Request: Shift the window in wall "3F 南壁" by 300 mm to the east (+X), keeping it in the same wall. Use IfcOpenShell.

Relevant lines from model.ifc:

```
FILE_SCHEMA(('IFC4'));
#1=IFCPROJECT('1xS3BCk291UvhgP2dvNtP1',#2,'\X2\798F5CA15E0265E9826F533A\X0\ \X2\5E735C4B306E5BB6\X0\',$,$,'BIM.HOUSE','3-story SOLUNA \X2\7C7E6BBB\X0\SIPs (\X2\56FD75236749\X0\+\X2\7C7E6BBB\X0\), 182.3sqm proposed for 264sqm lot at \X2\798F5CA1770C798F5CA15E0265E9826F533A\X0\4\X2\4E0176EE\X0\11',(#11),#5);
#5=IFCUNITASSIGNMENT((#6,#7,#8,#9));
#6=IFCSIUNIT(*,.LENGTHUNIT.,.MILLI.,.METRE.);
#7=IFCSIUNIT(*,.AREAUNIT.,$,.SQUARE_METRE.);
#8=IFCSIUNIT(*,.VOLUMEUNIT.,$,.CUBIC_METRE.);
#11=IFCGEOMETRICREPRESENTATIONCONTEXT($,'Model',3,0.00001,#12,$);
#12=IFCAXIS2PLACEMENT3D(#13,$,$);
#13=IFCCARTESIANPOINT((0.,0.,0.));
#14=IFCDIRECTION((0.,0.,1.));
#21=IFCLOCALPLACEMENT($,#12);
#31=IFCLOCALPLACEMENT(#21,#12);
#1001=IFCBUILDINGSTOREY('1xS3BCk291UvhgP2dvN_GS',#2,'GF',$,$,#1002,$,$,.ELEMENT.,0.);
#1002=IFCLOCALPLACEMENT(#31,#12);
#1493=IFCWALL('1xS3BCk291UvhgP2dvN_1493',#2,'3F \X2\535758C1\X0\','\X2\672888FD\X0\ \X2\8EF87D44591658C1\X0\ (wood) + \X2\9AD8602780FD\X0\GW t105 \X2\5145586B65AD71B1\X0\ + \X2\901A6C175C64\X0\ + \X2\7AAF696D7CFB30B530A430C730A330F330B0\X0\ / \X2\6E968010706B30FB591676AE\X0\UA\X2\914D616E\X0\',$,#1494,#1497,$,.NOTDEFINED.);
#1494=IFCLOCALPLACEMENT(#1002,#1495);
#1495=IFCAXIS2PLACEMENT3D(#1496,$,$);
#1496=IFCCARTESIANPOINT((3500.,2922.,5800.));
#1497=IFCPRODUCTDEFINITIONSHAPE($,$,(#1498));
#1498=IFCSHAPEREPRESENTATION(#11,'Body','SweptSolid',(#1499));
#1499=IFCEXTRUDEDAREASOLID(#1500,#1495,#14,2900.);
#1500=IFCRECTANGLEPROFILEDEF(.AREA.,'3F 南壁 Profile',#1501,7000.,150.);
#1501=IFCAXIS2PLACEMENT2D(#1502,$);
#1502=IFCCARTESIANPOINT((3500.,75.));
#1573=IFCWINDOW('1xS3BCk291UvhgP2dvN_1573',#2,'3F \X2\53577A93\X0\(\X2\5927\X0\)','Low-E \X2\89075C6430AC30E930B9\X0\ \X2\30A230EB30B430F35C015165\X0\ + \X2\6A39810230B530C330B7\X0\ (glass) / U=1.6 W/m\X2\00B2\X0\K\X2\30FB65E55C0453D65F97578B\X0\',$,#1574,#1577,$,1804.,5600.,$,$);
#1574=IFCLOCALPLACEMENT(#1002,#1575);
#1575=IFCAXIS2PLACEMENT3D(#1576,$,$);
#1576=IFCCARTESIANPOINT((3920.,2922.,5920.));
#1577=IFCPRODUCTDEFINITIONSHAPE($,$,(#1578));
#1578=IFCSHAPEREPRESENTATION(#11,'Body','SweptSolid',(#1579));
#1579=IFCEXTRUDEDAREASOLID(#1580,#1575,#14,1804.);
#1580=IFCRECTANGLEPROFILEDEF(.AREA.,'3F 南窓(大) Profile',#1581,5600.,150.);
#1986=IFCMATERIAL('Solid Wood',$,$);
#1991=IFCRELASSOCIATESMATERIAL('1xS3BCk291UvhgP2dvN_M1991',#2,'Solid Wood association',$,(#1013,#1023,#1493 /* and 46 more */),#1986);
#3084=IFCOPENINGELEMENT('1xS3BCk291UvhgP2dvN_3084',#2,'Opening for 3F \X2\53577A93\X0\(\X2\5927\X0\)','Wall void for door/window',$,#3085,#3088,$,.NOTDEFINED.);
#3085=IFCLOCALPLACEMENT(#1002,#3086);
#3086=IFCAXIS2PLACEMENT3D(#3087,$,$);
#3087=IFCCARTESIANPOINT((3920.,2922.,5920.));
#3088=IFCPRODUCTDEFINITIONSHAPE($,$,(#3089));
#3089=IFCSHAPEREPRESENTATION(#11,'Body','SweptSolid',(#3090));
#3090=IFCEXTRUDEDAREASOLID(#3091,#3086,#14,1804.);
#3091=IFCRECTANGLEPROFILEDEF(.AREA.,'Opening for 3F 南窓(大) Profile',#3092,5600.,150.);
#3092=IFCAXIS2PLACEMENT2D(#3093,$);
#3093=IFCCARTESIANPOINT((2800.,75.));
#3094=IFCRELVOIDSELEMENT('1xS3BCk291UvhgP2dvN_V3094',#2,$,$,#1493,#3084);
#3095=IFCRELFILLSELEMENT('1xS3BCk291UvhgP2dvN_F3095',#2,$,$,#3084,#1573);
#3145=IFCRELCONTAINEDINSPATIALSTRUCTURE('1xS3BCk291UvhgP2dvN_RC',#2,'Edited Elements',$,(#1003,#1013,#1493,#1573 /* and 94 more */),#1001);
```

```python
import ifcopenshell
import ifcopenshell.api.geometry
import ifcopenshell.util.placement
import ifcopenshell.util.unit

model = ifcopenshell.open("model.ifc")
unit_scale = ifcopenshell.util.unit.calculate_unit_scale(model)

window = model.by_id(1573)
opening = window.FillsVoids[0].RelatingOpeningElement
wall = opening.VoidsElements[0].RelatingBuildingElement

wall_matrix = ifcopenshell.util.placement.get_local_placement(wall.ObjectPlacement)
shift = wall_matrix[:3, 0] * 0.3 / unit_scale
before = ifcopenshell.util.placement.get_local_placement(window.ObjectPlacement)[:3, 3].copy()

# The window is not placed relative to its opening, so move both.
for product in (opening, window):
    matrix = ifcopenshell.util.placement.get_local_placement(product.ObjectPlacement)
    matrix[:3, 3] += shift
    ifcopenshell.api.geometry.edit_object_placement(model, product=product, matrix=matrix, is_si=False)

after = ifcopenshell.util.placement.get_local_placement(window.ObjectPlacement)[:3, 3]
print("window moved by", (after - before).round(3) + 0.0)

model.write("model-out.ifc")
```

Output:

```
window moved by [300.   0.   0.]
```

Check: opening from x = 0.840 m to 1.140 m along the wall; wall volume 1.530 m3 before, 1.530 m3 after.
